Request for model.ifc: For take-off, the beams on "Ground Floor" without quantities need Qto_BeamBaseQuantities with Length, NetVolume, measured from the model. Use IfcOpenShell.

First a look at what the model holds.

```python
import ifcopenshell
import ifcopenshell.util.element
import ifcopenshell.util.unit

model = ifcopenshell.open("model.ifc")
print(model.schema)
for unit_type in ("LENGTHUNIT", "AREAUNIT", "VOLUMEUNIT"):
    print(unit_type, ifcopenshell.util.unit.calculate_unit_scale(model, unit_type))
storey = next(s for s in model.by_type("IfcBuildingStorey") if s.Name == "Ground Floor")
beams = [e for e in ifcopenshell.util.element.get_decomposition(storey) if e.is_a("IfcBeam")]
for e in sorted(beams, key=lambda e: e.id()):
    print(e.id(), e.is_a(), e.Name, list(ifcopenshell.util.element.get_psets(e, qtos_only=True)), sep=" | ")
```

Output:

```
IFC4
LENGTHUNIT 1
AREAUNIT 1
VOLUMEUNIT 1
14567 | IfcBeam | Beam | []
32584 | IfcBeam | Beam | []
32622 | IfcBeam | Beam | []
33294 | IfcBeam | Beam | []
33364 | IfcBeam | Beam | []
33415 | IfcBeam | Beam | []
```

```python
import ifcopenshell
import ifcopenshell.api.pset
import ifcopenshell.geom
import ifcopenshell.util.element
import ifcopenshell.util.shape
import ifcopenshell.util.unit

model = ifcopenshell.open("model.ifc")
unit_scale = ifcopenshell.util.unit.calculate_unit_scale(model)
volume_scale = ifcopenshell.util.unit.calculate_unit_scale(model, "VOLUMEUNIT")
settings = ifcopenshell.geom.settings()

storey = next(s for s in model.by_type("IfcBuildingStorey") if s.Name == "Ground Floor")
beams = [e for e in ifcopenshell.util.element.get_decomposition(storey) if e.is_a("IfcBeam")]

for e in sorted(beams, key=lambda e: e.id()):
    if ifcopenshell.util.element.get_psets(e, qtos_only=True, should_inherit=False):
        continue
    # Geometry comes back in metres, in the element's own axes.
    shape = ifcopenshell.geom.create_shape(settings, e)
    values = {
        "Length": ifcopenshell.util.shape.get_max_xyz(shape.geometry) / unit_scale,
        "NetVolume": ifcopenshell.util.shape.get_volume(shape.geometry) / volume_scale,
    }
    qto = ifcopenshell.api.pset.add_qto(model, product=e, name="Qto_BeamBaseQuantities")
    ifcopenshell.api.pset.edit_qto(model, qto=qto, properties=values)
    print(e.id(), {k: round(v, 3) for k, v in values.items()})

model.write("model_edited.ifc")
```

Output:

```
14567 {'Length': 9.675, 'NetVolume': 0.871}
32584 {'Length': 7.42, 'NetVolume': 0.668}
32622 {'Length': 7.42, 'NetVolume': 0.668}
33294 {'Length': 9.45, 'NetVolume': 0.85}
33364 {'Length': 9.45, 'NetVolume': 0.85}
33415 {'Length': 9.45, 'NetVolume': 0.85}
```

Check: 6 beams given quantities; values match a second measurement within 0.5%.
